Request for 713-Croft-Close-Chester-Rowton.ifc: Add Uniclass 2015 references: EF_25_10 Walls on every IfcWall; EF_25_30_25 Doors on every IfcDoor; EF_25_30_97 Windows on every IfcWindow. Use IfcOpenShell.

First a look at what the model holds.

```python
import ifcopenshell

model = ifcopenshell.open("713-Croft-Close-Chester-Rowton.ifc")
print(model.schema)
print("classifications:", [c.Name for c in model.by_type("IfcClassification")])
for ifc_class in ("IfcDoor", "IfcRoof", "IfcStair", "IfcWall", "IfcWindow"):
    print(ifc_class, len(model.by_type(ifc_class)))
```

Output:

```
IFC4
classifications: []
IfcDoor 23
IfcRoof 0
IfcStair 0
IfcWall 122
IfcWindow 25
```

```python
import ifcopenshell
import ifcopenshell.api.classification

model = ifcopenshell.open("713-Croft-Close-Chester-Rowton.ifc")

system = ifcopenshell.api.classification.add_classification(model, classification="Uniclass 2015")

codes = {
    "IfcWall": ("EF_25_10", "Walls"),
    "IfcDoor": ("EF_25_30_25", "Doors"),
    "IfcWindow": ("EF_25_30_97", "Windows"),
}
for ifc_class, (code, name) in codes.items():
    products = model.by_type(ifc_class)
    ifcopenshell.api.classification.add_reference(
        model, products=products, classification=system, identification=code, name=name
    )
    print(code, len(products))

model.write("713-Croft-Close-Chester-Rowton_updated.ifc")
```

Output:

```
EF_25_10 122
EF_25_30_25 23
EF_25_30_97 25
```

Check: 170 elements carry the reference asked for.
